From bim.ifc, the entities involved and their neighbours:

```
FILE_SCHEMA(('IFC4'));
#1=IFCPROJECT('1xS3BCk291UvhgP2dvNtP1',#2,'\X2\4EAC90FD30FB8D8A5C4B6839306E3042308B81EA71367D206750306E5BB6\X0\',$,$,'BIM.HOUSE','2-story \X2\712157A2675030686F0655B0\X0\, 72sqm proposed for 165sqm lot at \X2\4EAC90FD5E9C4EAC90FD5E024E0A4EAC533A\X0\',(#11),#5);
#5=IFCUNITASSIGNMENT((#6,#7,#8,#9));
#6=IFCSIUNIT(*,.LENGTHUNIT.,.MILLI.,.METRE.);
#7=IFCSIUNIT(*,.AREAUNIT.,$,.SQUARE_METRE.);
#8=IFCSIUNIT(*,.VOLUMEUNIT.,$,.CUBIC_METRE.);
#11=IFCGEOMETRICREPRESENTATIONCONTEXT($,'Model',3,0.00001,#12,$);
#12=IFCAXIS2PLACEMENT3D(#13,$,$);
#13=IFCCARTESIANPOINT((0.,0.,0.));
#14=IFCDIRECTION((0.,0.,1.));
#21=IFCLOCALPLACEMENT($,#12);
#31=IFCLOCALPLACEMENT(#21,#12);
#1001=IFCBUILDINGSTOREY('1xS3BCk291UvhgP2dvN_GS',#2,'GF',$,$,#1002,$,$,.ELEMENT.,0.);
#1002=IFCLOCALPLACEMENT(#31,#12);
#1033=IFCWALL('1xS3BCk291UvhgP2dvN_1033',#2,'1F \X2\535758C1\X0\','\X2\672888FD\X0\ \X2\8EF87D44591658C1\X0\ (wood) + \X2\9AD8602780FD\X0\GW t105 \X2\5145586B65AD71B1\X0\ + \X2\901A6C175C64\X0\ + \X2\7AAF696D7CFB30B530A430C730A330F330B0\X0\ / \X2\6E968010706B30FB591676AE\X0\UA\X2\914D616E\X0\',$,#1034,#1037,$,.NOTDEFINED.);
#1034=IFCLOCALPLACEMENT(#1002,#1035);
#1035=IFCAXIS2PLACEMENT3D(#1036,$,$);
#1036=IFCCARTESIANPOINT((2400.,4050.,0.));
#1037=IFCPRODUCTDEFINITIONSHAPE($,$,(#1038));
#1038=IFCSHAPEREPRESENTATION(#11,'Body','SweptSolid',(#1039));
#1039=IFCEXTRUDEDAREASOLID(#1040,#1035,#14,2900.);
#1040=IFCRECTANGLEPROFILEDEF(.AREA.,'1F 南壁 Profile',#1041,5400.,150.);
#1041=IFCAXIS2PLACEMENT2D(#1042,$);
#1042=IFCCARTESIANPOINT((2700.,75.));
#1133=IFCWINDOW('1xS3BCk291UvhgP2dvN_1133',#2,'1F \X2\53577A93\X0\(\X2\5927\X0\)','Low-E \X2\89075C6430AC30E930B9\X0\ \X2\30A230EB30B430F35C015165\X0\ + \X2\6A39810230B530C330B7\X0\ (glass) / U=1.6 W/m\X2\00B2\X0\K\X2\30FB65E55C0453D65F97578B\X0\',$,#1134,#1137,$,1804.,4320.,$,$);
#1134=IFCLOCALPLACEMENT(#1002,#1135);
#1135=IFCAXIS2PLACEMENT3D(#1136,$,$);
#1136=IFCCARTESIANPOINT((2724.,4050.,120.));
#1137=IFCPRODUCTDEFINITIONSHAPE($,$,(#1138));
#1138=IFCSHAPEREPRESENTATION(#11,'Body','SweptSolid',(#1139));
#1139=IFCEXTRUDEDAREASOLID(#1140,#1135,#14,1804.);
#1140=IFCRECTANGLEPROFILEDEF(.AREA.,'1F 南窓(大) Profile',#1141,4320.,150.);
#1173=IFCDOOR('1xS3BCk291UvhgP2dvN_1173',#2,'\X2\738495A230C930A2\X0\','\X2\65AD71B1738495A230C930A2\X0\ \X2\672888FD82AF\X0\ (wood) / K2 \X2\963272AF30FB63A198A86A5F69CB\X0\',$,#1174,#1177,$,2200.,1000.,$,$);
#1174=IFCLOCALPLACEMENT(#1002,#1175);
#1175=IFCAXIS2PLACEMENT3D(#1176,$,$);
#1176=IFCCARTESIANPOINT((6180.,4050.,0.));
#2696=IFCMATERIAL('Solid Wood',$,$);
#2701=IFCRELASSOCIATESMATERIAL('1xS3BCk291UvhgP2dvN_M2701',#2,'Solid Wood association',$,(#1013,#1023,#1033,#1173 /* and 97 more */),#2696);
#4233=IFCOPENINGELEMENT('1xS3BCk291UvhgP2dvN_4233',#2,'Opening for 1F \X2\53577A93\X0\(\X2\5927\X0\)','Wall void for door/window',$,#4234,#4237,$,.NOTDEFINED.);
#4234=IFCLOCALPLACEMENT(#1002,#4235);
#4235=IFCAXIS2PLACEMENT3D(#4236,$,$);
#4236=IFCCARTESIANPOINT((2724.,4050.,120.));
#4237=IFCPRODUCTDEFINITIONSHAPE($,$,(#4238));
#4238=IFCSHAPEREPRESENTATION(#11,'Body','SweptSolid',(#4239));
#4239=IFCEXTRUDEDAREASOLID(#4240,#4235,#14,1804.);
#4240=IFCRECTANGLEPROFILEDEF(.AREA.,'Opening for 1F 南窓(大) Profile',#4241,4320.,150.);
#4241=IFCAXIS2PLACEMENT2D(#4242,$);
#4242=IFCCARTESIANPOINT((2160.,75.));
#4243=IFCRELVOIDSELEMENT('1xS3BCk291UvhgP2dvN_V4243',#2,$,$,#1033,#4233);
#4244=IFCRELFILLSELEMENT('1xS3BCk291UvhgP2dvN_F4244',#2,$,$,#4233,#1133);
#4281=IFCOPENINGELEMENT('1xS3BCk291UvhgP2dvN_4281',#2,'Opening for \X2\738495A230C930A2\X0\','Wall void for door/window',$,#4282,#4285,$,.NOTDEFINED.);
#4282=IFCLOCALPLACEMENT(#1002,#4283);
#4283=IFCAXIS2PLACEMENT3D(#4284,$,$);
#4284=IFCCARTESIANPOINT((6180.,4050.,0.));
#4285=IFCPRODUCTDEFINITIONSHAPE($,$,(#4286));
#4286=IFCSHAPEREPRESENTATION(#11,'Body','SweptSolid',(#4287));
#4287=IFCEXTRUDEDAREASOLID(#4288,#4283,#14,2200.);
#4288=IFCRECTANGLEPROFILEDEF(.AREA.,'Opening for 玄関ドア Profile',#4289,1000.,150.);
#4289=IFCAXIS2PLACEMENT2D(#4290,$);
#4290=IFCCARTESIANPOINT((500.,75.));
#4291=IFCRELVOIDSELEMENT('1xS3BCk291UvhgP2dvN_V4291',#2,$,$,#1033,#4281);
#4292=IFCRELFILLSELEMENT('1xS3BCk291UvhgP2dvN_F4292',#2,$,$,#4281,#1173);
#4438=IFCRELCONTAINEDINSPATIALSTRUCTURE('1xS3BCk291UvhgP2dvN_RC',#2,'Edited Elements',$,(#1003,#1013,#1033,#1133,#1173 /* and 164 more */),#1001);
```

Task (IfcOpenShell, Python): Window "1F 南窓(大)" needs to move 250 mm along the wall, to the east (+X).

```python
import ifcopenshell
import ifcopenshell.api.geometry
import ifcopenshell.util.placement
import ifcopenshell.util.unit

model = ifcopenshell.open("bim.ifc")
unit_scale = ifcopenshell.util.unit.calculate_unit_scale(model)

window = model.by_guid("1xS3BCk291UvhgP2dvN_1133")
opening = window.FillsVoids[0].RelatingOpeningElement
wall = opening.VoidsElements[0].RelatingBuildingElement

wall_matrix = ifcopenshell.util.placement.get_local_placement(wall.ObjectPlacement)
shift = wall_matrix[:3, 0] * 0.25 / unit_scale
before = ifcopenshell.util.placement.get_local_placement(window.ObjectPlacement)[:3, 3].copy()

# The window is not placed relative to its opening, so move both.
for product in (opening, window):
    matrix = ifcopenshell.util.placement.get_local_placement(product.ObjectPlacement)
    matrix[:3, 3] += shift
    ifcopenshell.api.geometry.edit_object_placement(model, product=product, matrix=matrix, is_si=False)

after = ifcopenshell.util.placement.get_local_placement(window.ObjectPlacement)[:3, 3]
print("window moved by", (after - before).round(3) + 0.0)

model.write("bim_rev.ifc")
```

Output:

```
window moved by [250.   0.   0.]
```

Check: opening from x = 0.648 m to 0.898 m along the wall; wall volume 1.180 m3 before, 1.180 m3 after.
